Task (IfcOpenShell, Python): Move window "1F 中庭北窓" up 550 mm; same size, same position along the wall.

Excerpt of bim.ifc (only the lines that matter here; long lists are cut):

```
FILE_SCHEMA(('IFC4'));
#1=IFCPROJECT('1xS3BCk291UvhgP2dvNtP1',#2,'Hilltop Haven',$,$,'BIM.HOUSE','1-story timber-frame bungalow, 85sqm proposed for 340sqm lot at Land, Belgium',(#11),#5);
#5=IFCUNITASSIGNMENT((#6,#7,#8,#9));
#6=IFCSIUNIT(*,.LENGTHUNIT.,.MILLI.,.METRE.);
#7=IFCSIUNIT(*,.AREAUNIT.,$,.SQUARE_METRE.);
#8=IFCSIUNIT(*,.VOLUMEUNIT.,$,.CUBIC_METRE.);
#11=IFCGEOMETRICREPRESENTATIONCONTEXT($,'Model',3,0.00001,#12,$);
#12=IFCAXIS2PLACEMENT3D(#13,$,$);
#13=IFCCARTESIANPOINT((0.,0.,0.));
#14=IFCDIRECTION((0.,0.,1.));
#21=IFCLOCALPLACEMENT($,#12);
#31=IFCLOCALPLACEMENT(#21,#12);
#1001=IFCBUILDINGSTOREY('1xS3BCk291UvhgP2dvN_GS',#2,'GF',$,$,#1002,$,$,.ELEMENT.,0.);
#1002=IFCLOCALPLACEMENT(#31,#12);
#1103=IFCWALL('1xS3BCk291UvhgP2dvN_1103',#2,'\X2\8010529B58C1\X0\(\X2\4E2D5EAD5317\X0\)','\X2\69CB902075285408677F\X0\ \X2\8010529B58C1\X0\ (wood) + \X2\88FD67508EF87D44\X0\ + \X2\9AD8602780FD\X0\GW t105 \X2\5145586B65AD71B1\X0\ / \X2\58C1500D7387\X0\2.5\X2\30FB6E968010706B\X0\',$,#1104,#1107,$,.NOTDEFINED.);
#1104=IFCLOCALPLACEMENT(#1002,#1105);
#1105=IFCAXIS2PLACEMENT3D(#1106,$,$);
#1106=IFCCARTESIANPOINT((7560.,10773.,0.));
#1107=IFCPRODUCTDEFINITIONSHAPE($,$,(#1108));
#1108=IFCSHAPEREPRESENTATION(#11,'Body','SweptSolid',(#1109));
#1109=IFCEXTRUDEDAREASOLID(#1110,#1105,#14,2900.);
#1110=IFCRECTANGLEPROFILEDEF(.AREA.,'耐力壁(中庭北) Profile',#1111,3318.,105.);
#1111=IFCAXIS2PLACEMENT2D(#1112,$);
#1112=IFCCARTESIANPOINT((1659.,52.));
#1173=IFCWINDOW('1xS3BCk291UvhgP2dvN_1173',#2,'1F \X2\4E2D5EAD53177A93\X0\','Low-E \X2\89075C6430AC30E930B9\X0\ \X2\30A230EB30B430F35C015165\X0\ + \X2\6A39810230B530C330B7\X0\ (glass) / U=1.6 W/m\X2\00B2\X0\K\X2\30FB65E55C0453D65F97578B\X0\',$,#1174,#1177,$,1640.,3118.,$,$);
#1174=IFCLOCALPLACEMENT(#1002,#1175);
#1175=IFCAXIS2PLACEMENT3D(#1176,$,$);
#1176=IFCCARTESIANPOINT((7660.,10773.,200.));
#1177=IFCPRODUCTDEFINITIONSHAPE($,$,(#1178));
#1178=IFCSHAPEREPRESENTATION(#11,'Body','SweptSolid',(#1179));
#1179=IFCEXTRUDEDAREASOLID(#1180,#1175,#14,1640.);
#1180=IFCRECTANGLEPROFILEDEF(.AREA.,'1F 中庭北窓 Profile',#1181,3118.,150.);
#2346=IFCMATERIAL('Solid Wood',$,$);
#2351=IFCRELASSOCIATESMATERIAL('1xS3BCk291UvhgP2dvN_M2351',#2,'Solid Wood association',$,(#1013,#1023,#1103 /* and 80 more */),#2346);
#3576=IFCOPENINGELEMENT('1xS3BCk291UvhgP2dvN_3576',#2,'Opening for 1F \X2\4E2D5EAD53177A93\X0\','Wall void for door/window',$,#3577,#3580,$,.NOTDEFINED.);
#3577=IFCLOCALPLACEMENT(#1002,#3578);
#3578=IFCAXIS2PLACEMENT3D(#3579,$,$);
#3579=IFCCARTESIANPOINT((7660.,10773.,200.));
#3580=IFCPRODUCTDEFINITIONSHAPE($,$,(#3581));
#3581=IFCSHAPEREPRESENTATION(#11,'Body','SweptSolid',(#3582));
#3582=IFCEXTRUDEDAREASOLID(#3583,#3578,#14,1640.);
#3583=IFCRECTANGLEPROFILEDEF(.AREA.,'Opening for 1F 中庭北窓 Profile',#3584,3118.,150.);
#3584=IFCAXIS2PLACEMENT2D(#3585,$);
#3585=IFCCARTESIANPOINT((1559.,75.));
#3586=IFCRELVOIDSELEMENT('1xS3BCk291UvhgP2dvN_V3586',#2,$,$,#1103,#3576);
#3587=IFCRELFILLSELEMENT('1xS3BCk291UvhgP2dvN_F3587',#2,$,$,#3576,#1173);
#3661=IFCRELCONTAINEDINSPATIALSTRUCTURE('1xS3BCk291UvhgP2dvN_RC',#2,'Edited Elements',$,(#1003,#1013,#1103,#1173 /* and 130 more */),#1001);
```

```python
import numpy as np
import ifcopenshell
import ifcopenshell.api.geometry
import ifcopenshell.util.placement
import ifcopenshell.util.unit

model = ifcopenshell.open("bim.ifc")
unit_scale = ifcopenshell.util.unit.calculate_unit_scale(model)

window = model.by_id(1173)
opening = window.FillsVoids[0].RelatingOpeningElement
dz = 550.0

shift = np.array([0.0, 0.0, dz])
# The window is not placed relative to its opening, so move both.
for product in (opening, window):
    matrix = ifcopenshell.util.placement.get_local_placement(product.ObjectPlacement)
    matrix[:3, 3] += shift
    ifcopenshell.api.geometry.edit_object_placement(model, product=product, matrix=matrix, is_si=False)

print(f"moved by {dz * unit_scale:+.3f} m")

model.write("bim_updated.ifc")
```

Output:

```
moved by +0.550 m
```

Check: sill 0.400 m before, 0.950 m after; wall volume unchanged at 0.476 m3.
